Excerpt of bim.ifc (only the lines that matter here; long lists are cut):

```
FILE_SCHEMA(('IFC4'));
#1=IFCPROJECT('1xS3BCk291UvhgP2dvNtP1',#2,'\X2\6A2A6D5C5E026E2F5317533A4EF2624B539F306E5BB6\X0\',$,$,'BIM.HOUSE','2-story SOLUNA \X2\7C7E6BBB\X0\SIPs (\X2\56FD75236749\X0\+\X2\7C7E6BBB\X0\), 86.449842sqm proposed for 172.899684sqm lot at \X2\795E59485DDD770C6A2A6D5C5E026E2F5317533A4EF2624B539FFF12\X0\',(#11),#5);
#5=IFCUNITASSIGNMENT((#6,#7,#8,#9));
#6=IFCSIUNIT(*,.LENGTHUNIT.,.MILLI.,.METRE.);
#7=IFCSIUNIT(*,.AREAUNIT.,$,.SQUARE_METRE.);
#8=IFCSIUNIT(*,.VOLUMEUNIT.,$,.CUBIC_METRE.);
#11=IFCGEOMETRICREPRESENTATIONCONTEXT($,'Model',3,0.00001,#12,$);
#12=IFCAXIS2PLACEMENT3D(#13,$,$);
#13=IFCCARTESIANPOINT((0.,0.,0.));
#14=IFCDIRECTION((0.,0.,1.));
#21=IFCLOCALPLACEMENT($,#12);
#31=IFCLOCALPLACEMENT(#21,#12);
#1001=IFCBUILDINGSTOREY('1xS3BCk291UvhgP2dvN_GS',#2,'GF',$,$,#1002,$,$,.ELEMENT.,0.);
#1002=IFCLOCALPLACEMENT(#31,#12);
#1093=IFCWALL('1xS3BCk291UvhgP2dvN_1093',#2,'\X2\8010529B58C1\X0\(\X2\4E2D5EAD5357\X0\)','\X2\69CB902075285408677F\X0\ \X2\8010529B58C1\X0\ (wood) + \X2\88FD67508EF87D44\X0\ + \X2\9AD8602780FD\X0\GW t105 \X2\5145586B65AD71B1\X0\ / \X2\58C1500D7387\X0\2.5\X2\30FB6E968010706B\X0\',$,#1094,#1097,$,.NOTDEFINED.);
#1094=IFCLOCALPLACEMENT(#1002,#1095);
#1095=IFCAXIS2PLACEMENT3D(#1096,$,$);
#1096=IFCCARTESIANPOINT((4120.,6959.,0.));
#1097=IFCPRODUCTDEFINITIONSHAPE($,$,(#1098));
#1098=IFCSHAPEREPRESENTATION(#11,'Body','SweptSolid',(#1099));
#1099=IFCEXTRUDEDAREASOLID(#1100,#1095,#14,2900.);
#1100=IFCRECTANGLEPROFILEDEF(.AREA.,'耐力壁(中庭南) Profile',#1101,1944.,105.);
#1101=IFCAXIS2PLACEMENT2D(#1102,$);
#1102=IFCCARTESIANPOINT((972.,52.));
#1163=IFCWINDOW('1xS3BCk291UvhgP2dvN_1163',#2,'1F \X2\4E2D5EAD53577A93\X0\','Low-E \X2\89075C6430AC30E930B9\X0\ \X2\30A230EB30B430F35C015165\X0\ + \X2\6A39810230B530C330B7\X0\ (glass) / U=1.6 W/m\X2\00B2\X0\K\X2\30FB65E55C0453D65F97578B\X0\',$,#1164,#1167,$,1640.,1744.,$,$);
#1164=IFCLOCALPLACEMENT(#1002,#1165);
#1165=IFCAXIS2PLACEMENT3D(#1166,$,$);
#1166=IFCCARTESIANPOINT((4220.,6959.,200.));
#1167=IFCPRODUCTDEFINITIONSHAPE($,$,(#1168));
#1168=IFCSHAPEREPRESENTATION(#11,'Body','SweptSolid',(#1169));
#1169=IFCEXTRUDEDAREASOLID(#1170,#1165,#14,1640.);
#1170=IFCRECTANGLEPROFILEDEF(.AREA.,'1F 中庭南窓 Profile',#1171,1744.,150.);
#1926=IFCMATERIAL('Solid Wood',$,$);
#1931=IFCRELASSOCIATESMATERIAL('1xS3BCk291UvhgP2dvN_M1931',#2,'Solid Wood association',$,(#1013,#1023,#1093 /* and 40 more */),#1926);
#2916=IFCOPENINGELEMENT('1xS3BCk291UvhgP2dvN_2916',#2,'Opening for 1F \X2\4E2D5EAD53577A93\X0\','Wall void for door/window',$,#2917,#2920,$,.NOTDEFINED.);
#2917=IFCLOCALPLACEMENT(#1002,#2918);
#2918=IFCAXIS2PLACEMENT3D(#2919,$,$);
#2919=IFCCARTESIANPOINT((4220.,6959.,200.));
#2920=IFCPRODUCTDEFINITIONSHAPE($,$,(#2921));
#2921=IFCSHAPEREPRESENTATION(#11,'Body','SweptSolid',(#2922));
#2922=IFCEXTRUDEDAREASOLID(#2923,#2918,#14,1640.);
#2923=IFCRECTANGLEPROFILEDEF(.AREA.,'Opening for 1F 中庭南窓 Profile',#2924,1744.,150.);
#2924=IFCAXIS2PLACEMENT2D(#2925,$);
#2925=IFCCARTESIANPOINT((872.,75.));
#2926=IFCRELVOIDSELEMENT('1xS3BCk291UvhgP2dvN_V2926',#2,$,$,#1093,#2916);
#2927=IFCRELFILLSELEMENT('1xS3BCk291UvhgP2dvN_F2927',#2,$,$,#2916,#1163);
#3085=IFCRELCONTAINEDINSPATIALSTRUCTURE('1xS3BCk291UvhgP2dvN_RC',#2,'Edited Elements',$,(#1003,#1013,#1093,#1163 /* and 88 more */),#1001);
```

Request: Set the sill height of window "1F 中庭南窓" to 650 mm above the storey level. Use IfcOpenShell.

```python
import numpy as np
import ifcopenshell
import ifcopenshell.api.geometry
import ifcopenshell.geom
import ifcopenshell.util.element
import ifcopenshell.util.placement
import ifcopenshell.util.shape
import ifcopenshell.util.unit

model = ifcopenshell.open("bim.ifc")
unit_scale = ifcopenshell.util.unit.calculate_unit_scale(model)

window = model.by_id(1163)
opening = window.FillsVoids[0].RelatingOpeningElement
storey = ifcopenshell.util.element.get_container(window, ifc_class="IfcBuildingStorey")
level = ifcopenshell.util.placement.get_local_placement(storey.ObjectPlacement)[2, 3]

# The opening's origin need not be at the sill, so measure its lowest point.
shape = ifcopenshell.geom.create_shape(ifcopenshell.geom.settings(), opening)
bottom = ifcopenshell.util.shape.get_shape_bottom_elevation(shape, shape.geometry) / unit_scale
dz = level + 650.0 - bottom

shift = np.array([0.0, 0.0, dz])
# The window is not placed relative to its opening, so move both.
for product in (opening, window):
    matrix = ifcopenshell.util.placement.get_local_placement(product.ObjectPlacement)
    matrix[:3, 3] += shift
    ifcopenshell.api.geometry.edit_object_placement(model, product=product, matrix=matrix, is_si=False)

print(f"moved by {dz * unit_scale:+.3f} m")

model.write("bim_v2.ifc")
```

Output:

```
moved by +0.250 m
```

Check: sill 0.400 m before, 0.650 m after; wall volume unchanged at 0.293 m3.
